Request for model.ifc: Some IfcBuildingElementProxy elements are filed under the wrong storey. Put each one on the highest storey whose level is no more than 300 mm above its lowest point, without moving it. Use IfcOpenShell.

First a look at what the model holds.

```python
import ifcopenshell
import ifcopenshell.util.element
import ifcopenshell.util.placement

model = ifcopenshell.open("model.ifc")
print(model.schema)
for storey in model.by_type("IfcBuildingStorey"):
    level = ifcopenshell.util.placement.get_storey_elevation(storey)
    count = sum(e.is_a("IfcBuildingElementProxy") for e in ifcopenshell.util.element.get_contained(storey))
    print(storey.id(), storey.Name, round(level, 3), count, sep=" | ")
```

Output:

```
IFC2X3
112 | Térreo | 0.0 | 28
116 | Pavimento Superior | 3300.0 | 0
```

```python
import ifcopenshell
import ifcopenshell.api.spatial
import ifcopenshell.geom
import ifcopenshell.util.element
import ifcopenshell.util.placement
import ifcopenshell.util.shape
import ifcopenshell.util.unit

model = ifcopenshell.open("model.ifc")
unit_scale = ifcopenshell.util.unit.calculate_unit_scale(model)
settings = ifcopenshell.geom.settings()

levels = sorted(
    ((ifcopenshell.util.placement.get_storey_elevation(s) * unit_scale, s) for s in model.by_type("IfcBuildingStorey")),
    key=lambda pair: pair[0],
)

for e in model.by_type("IfcBuildingElementProxy"):
    current = e.ContainedInStructure[0].RelatingStructure if e.ContainedInStructure else None
    if current is None or not current.is_a("IfcBuildingStorey"):
        continue
    shape = ifcopenshell.geom.create_shape(settings, e)
    bottom = ifcopenshell.util.shape.get_shape_bottom_elevation(shape, shape.geometry)
    below = [s for level, s in levels if level <= bottom + 0.3]
    storey = below[-1] if below else levels[0][1]
    if storey != current:
        # assign_container keeps the world position.
        ifcopenshell.api.spatial.assign_container(model, products=[e], relating_structure=storey)
        print(e.id(), current.Name, "->", storey.Name)

model.write("model_v2.ifc")
```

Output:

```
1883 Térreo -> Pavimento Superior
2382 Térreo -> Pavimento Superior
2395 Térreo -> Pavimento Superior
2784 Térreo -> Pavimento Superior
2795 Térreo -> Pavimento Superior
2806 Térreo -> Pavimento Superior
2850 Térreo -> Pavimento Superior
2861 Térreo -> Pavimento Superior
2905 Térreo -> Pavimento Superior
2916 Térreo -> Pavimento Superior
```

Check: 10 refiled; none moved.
